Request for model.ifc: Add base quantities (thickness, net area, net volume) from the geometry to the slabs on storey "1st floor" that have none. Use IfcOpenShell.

First a look at what the model holds.

```python
import ifcopenshell
import ifcopenshell.util.element
import ifcopenshell.util.unit

model = ifcopenshell.open("model.ifc")
print(model.schema)
for unit_type in ("LENGTHUNIT", "AREAUNIT", "VOLUMEUNIT"):
    print(unit_type, ifcopenshell.util.unit.calculate_unit_scale(model, unit_type))
storey = next(s for s in model.by_type("IfcBuildingStorey") if s.Name == "1st floor")
slabs = [e for e in ifcopenshell.util.element.get_decomposition(storey) if e.is_a("IfcSlab")]
for e in sorted(slabs, key=lambda e: e.id()):
    print(e.id(), e.is_a(), e.Name, list(ifcopenshell.util.element.get_psets(e, qtos_only=True)), sep=" | ")
```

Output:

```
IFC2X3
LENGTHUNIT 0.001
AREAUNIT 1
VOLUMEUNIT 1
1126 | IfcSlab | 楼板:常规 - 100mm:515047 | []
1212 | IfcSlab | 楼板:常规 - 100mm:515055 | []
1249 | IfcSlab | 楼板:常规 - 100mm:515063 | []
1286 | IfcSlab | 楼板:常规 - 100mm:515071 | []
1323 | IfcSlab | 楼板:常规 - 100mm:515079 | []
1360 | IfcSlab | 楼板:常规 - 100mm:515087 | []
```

```python
import ifcopenshell
import ifcopenshell.api.pset
import ifcopenshell.geom
import ifcopenshell.util.element
import ifcopenshell.util.shape
import ifcopenshell.util.unit

model = ifcopenshell.open("model.ifc")
unit_scale = ifcopenshell.util.unit.calculate_unit_scale(model)
area_scale = ifcopenshell.util.unit.calculate_unit_scale(model, "AREAUNIT")
volume_scale = ifcopenshell.util.unit.calculate_unit_scale(model, "VOLUMEUNIT")
settings = ifcopenshell.geom.settings()

storey = next(s for s in model.by_type("IfcBuildingStorey") if s.Name == "1st floor")
slabs = [e for e in ifcopenshell.util.element.get_decomposition(storey) if e.is_a("IfcSlab")]

for e in sorted(slabs, key=lambda e: e.id()):
    if ifcopenshell.util.element.get_psets(e, qtos_only=True, should_inherit=False):
        continue
    # Geometry comes back in metres, in the element's own axes.
    shape = ifcopenshell.geom.create_shape(settings, e)
    values = {
        "Width": ifcopenshell.util.shape.get_z(shape.geometry) / unit_scale,
        "NetArea": ifcopenshell.util.shape.get_footprint_area(shape.geometry) / area_scale,
        "NetVolume": ifcopenshell.util.shape.get_volume(shape.geometry) / volume_scale,
    }
    qto = ifcopenshell.api.pset.add_qto(model, product=e, name="BaseQuantities")
    ifcopenshell.api.pset.edit_qto(model, qto=qto, properties=values)
    print(e.id(), {k: round(v, 3) for k, v in values.items()})

model.write("model_edited.ifc")
```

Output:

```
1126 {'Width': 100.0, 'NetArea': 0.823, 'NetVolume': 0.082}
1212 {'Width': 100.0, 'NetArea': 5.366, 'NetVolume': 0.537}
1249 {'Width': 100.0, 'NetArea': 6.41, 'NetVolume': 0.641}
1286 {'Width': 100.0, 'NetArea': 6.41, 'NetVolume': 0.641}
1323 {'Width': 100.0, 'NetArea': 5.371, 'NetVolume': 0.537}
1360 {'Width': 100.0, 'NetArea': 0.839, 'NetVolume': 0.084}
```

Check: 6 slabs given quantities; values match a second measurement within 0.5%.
